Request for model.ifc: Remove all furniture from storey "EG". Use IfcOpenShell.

First a look at what the model holds.

```python
import ifcopenshell
import ifcopenshell.util.element

model = ifcopenshell.open("model.ifc")
print(model.schema)
storey = next(s for s in model.by_type("IfcBuildingStorey") if s.Name == "EG")
furniture = [e for e in ifcopenshell.util.element.get_decomposition(storey) if e.is_a("IfcFurnishingElement")]
seen = {}
for e in furniture:
    element_type = ifcopenshell.util.element.get_type(e)
    name = element_type.Name if element_type not in (None, e) else None
    seen[name] = seen.get(name, 0) + 1
for name, count in sorted(seen.items(), key=str):
    print(count, "x", name)
```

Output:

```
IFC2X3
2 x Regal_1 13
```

```python
import ifcopenshell
import ifcopenshell.api.root
import ifcopenshell.util.element

model = ifcopenshell.open("model.ifc")

storey = next(s for s in model.by_type("IfcBuildingStorey") if s.Name == "EG")
furniture = [e for e in ifcopenshell.util.element.get_decomposition(storey) if e.is_a("IfcFurnishingElement")]

for e in furniture:
    ifcopenshell.api.root.remove_product(model, product=e)
print(len(furniture), "removed")

model.write("model_edited.ifc")
```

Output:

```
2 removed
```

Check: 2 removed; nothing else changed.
